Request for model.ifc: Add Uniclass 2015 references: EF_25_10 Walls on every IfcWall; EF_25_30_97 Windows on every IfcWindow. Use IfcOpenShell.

First a look at what the model holds.

```python
import ifcopenshell

model = ifcopenshell.open("model.ifc")
print(model.schema)
print("classifications:", [c.Name for c in model.by_type("IfcClassification")])
for ifc_class in ("IfcDoor", "IfcRoof", "IfcStair", "IfcWall", "IfcWindow"):
    print(ifc_class, len(model.by_type(ifc_class)))
```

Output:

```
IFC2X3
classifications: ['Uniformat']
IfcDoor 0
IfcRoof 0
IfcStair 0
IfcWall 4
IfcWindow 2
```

```python
import ifcopenshell
import ifcopenshell.api.classification

model = ifcopenshell.open("model.ifc")

# IFC2X3 requires Source and Edition and has no link from the project to the system.
system = model.create_entity("IfcClassification", Source="NBS", Edition="2015", Name="Uniclass 2015")

codes = {
    "IfcWall": ("EF_25_10", "Walls"),
    "IfcWindow": ("EF_25_30_97", "Windows"),
}
for ifc_class, (code, name) in codes.items():
    products = model.by_type(ifc_class)
    ifcopenshell.api.classification.add_reference(
        model, products=products, classification=system, identification=code, name=name
    )
    print(code, len(products))

model.write("model-out.ifc")
```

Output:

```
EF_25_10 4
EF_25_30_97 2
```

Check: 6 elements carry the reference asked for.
